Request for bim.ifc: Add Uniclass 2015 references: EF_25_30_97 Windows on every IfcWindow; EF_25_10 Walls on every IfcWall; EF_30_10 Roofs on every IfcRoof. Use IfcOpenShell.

First a look at what the model holds.

```python
import ifcopenshell

model = ifcopenshell.open("bim.ifc")
print(model.schema)
print("classifications:", [c.Name for c in model.by_type("IfcClassification")])
for ifc_class in ("IfcDoor", "IfcRoof", "IfcStair", "IfcWall", "IfcWindow"):
    print(ifc_class, len(model.by_type(ifc_class)))
```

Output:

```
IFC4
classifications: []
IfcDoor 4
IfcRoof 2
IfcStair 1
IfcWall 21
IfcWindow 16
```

```python
import ifcopenshell
import ifcopenshell.api.classification

model = ifcopenshell.open("bim.ifc")

system = ifcopenshell.api.classification.add_classification(model, classification="Uniclass 2015")

codes = {
    "IfcWindow": ("EF_25_30_97", "Windows"),
    "IfcWall": ("EF_25_10", "Walls"),
    "IfcRoof": ("EF_30_10", "Roofs"),
}
for ifc_class, (code, name) in codes.items():
    products = model.by_type(ifc_class)
    ifcopenshell.api.classification.add_reference(
        model, products=products, classification=system, identification=code, name=name
    )
    print(code, len(products))

model.write("bim_edited.ifc")
```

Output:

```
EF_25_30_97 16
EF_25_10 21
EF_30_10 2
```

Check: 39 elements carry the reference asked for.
